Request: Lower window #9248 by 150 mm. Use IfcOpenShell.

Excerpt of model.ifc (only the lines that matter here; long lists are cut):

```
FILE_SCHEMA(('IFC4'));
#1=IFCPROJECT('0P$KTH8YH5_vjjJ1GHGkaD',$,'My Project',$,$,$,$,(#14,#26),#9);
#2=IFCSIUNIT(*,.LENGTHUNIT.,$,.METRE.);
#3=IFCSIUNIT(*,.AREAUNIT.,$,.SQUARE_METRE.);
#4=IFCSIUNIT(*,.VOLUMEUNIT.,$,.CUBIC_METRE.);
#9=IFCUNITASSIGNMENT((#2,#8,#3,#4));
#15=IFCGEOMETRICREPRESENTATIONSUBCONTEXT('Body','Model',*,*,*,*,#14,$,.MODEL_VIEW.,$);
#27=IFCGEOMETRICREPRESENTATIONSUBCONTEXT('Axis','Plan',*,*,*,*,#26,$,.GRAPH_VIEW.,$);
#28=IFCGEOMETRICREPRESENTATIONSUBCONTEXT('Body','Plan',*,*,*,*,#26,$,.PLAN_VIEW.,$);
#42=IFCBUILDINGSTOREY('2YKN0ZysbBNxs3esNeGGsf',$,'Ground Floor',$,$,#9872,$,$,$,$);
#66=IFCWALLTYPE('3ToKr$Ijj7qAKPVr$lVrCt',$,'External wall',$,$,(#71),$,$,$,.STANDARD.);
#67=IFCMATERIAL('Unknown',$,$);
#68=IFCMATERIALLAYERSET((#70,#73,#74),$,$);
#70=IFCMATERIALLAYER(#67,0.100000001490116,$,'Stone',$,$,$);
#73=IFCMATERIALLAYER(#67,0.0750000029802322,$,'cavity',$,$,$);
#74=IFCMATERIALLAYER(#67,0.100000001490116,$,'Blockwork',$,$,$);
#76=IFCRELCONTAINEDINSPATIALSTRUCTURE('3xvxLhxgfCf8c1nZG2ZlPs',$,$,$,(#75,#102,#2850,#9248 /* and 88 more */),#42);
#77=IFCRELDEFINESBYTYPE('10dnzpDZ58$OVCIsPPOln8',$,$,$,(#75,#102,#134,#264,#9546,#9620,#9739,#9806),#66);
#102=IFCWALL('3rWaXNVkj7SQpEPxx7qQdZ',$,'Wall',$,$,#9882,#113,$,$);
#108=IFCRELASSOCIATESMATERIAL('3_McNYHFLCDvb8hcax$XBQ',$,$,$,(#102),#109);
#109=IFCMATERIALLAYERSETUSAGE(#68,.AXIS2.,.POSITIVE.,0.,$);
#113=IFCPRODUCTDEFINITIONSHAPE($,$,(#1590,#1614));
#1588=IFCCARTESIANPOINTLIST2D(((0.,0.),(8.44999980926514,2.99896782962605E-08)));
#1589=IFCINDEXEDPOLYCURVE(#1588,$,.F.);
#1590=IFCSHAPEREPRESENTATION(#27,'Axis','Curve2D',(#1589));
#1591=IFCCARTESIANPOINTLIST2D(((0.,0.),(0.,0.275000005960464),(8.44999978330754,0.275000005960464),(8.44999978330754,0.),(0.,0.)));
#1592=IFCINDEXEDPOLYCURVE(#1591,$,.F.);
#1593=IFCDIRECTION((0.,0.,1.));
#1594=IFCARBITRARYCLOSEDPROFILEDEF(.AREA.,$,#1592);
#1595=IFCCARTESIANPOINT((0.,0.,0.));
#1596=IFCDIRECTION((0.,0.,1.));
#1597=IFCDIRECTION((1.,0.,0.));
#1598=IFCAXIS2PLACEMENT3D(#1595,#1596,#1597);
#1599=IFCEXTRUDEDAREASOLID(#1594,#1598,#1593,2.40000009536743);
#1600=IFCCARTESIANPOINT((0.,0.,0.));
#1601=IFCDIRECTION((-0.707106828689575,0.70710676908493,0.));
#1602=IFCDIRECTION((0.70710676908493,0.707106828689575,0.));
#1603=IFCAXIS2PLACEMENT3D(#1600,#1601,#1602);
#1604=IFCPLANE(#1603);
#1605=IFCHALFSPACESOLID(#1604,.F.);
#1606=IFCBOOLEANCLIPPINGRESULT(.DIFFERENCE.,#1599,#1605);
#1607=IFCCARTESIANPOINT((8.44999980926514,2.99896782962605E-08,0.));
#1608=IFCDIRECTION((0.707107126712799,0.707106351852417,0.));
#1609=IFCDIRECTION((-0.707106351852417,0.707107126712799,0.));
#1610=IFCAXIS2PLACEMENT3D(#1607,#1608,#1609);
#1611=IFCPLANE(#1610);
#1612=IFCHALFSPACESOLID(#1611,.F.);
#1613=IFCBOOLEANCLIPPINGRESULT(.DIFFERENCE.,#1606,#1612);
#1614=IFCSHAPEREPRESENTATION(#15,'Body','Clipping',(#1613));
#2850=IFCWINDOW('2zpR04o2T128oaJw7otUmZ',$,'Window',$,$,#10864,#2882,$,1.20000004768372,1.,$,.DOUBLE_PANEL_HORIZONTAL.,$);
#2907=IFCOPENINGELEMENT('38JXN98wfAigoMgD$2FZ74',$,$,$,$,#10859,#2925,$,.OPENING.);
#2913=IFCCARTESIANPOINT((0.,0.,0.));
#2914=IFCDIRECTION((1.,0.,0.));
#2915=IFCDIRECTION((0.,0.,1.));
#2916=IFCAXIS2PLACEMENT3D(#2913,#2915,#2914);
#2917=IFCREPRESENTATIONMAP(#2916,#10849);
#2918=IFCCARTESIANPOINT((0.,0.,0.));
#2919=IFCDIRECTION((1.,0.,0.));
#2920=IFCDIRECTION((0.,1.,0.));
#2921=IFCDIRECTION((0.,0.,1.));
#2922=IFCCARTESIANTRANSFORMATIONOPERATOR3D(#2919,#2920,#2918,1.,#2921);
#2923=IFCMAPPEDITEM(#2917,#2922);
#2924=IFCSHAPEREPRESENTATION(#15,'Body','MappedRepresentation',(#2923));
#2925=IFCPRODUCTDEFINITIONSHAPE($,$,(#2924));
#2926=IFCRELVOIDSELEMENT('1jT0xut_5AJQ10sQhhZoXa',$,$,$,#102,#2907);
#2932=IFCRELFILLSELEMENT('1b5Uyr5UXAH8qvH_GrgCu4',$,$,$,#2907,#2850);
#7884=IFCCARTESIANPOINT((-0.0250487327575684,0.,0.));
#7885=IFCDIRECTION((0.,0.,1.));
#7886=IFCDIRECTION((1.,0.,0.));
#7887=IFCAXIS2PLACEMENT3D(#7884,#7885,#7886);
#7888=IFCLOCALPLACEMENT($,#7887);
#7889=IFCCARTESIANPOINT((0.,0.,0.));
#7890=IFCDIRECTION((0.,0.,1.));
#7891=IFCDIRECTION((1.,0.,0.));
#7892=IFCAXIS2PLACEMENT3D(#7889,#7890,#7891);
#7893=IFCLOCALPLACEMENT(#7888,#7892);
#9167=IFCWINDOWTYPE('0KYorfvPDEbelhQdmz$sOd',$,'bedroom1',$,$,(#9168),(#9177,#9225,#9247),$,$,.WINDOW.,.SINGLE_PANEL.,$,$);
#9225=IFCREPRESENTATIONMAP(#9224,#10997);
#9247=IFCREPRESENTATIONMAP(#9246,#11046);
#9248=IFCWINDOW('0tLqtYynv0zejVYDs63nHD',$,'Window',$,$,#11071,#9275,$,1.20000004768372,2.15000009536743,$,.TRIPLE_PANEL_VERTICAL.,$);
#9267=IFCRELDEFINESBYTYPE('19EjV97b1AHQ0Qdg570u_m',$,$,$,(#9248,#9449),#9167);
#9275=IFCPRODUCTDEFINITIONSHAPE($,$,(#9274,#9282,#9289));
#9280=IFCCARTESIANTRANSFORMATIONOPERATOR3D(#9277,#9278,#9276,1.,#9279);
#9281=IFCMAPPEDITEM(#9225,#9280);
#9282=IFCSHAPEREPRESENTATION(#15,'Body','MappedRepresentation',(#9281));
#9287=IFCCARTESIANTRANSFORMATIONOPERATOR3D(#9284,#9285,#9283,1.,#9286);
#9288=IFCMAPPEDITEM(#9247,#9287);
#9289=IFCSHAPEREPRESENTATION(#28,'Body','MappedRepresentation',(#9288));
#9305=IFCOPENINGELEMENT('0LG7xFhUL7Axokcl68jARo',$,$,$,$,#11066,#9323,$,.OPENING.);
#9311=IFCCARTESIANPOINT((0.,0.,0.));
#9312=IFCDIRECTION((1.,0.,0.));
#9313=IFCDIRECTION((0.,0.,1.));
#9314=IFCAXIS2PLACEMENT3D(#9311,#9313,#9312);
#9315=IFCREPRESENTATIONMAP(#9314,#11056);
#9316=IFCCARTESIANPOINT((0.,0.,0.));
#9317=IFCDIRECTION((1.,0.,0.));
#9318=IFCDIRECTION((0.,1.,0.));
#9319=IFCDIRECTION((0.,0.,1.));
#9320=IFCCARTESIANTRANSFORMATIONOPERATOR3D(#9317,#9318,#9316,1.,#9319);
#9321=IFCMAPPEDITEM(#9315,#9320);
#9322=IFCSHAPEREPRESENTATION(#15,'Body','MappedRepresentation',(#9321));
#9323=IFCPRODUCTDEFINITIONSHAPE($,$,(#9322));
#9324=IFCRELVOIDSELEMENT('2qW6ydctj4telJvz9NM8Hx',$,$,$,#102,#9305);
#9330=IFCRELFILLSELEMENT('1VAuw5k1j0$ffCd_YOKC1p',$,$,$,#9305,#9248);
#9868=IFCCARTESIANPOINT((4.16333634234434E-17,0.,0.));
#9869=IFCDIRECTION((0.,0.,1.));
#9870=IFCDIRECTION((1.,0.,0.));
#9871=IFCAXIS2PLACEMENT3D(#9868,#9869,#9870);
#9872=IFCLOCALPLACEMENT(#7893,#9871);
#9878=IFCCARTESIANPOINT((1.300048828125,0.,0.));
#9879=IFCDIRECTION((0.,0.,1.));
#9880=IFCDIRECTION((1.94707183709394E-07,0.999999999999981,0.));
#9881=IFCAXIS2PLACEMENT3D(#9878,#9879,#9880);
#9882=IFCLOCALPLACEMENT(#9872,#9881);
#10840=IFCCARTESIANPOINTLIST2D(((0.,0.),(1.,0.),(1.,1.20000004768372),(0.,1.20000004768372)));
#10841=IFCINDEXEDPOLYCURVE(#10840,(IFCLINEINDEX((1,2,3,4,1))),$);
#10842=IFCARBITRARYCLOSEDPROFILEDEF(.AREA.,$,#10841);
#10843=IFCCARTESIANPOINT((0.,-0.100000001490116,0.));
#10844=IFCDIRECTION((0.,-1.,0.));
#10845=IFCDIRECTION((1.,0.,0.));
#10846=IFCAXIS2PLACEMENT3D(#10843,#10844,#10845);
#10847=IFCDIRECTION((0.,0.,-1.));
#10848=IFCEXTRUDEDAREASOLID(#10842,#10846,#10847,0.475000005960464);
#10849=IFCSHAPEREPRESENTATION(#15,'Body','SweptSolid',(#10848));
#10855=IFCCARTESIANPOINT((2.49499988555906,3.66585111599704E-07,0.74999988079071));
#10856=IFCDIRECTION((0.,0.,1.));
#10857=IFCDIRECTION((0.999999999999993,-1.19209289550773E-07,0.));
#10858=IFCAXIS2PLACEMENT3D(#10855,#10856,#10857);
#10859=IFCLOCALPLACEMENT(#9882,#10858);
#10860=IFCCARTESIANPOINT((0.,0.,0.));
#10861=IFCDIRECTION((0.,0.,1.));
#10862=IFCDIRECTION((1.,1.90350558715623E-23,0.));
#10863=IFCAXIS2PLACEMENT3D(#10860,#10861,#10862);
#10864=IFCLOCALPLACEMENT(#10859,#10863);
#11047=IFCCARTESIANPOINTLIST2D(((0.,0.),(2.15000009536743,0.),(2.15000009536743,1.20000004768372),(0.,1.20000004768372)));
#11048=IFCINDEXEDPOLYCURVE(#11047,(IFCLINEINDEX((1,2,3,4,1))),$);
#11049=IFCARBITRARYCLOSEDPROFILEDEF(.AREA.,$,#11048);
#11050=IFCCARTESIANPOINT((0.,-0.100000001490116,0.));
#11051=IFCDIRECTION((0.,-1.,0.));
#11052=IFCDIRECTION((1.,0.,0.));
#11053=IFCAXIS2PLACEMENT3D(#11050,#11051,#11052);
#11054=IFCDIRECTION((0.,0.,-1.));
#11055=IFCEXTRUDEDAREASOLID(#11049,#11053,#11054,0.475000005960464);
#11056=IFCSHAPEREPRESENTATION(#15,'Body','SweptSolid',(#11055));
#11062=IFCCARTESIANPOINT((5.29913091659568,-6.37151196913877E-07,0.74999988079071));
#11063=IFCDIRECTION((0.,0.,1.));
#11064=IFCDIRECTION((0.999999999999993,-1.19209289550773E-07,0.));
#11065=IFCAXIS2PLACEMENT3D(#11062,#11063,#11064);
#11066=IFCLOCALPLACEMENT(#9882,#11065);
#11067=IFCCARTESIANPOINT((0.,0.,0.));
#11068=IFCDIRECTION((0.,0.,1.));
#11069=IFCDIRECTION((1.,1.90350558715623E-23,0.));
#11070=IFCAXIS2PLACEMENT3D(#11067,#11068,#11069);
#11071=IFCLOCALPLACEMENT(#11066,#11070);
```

```python
import numpy as np
import ifcopenshell
import ifcopenshell.api.geometry
import ifcopenshell.util.placement
import ifcopenshell.util.unit

model = ifcopenshell.open("model.ifc")
unit_scale = ifcopenshell.util.unit.calculate_unit_scale(model)

window = model.by_guid("0tLqtYynv0zejVYDs63nHD")
opening = window.FillsVoids[0].RelatingOpeningElement
dz = -0.15

shift = np.array([0.0, 0.0, dz])
# The window is placed relative to its opening, so it follows when the opening moves.
matrix = ifcopenshell.util.placement.get_local_placement(opening.ObjectPlacement)
matrix[:3, 3] += shift
ifcopenshell.api.geometry.edit_object_placement(
    model, product=opening, matrix=matrix, is_si=False, should_transform_children=True
)

print(f"moved by {dz * unit_scale:+.3f} m")

model.write("model-out.ifc")
```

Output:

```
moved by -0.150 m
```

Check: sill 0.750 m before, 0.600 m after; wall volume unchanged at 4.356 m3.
